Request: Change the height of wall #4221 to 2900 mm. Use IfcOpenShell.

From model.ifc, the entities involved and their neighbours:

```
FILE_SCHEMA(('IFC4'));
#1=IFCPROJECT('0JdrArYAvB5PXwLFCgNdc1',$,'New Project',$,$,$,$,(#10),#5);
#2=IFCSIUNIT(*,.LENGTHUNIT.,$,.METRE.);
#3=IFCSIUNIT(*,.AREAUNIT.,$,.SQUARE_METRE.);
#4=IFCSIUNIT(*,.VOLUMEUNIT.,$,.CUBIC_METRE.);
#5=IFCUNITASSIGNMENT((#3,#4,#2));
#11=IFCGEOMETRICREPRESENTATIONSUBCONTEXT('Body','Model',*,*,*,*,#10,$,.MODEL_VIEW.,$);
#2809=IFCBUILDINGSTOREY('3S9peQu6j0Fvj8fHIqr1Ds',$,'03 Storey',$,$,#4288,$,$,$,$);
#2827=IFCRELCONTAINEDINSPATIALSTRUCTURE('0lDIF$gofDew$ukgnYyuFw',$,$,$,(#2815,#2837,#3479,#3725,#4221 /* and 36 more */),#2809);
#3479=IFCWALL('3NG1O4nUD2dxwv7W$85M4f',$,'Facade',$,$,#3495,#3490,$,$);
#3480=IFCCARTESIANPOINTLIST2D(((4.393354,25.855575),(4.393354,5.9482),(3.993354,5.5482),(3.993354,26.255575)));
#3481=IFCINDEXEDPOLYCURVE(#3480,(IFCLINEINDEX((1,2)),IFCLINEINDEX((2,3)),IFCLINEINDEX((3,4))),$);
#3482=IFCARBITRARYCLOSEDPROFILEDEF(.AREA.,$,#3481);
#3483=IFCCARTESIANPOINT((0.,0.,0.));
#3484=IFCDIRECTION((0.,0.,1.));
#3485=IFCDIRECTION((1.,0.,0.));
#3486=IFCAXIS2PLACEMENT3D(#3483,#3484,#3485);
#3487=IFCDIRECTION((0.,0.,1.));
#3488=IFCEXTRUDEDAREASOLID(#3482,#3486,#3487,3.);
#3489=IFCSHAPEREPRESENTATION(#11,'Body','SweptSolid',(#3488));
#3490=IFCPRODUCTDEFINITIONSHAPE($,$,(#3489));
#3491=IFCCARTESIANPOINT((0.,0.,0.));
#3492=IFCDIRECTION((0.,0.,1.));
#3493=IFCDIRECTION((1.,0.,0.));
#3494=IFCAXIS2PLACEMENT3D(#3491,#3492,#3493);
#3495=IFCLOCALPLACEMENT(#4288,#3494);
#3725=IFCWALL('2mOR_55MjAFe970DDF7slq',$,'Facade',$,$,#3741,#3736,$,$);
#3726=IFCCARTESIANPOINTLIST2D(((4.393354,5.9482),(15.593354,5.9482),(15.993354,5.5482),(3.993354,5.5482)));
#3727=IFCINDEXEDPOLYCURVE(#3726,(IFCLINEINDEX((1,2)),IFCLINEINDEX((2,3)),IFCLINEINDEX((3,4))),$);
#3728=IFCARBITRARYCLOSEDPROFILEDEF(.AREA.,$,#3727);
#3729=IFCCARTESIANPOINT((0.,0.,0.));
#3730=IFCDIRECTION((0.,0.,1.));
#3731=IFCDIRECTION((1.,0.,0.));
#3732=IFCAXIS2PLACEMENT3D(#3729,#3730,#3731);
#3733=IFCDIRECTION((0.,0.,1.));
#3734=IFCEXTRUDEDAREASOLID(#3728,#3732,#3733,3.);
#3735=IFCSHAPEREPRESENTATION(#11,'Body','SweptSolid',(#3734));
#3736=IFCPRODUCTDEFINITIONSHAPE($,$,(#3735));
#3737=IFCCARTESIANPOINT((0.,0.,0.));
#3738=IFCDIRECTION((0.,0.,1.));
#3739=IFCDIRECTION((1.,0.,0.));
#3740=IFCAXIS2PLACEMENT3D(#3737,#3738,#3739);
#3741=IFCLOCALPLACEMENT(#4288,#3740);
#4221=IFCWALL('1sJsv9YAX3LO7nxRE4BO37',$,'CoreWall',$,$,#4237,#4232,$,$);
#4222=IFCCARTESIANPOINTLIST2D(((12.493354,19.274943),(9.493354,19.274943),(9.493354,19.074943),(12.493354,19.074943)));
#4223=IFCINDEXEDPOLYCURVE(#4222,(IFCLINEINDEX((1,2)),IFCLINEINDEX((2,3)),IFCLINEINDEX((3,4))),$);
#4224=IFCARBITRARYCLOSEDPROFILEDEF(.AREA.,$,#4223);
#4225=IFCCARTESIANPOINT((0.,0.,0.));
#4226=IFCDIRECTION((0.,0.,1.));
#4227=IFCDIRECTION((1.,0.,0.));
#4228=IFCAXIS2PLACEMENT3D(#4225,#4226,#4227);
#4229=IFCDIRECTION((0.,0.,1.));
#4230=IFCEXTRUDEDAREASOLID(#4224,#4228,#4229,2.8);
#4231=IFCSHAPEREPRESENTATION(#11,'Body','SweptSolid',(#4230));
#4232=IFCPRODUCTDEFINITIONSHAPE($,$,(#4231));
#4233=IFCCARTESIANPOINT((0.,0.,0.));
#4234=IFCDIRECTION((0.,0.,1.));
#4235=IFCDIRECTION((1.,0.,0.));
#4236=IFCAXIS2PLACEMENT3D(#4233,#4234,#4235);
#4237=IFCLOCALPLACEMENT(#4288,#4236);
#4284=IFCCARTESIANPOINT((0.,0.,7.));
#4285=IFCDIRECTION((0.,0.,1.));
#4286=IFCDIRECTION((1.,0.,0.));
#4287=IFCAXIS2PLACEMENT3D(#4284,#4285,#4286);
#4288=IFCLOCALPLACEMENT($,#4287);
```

```python
import ifcopenshell
import ifcopenshell.geom
import ifcopenshell.util.representation
import ifcopenshell.util.shape
import ifcopenshell.util.unit

model = ifcopenshell.open("model.ifc")
unit_scale = ifcopenshell.util.unit.calculate_unit_scale(model)
settings = ifcopenshell.geom.settings()


def volume(element):
    """Net volume in cubic metres, openings subtracted."""
    shape = ifcopenshell.geom.create_shape(settings, element)
    return ifcopenshell.util.shape.get_volume(shape.geometry)


wall = model.by_guid("1sJsv9YAX3LO7nxRE4BO37")
before = volume(wall)

body = ifcopenshell.util.representation.get_representation(wall, "Model", "Body")
solid = body.Items[0]
old_height = solid.Depth
solid.Depth = 2.9 / unit_scale
after = volume(wall)

print(f"height {old_height:g} -> {solid.Depth:g}, volume {before:.3f} -> {after:.3f} m3")

model.write("model_updated.ifc")
```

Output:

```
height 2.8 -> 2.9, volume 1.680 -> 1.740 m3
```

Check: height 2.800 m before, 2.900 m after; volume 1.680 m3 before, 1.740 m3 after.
